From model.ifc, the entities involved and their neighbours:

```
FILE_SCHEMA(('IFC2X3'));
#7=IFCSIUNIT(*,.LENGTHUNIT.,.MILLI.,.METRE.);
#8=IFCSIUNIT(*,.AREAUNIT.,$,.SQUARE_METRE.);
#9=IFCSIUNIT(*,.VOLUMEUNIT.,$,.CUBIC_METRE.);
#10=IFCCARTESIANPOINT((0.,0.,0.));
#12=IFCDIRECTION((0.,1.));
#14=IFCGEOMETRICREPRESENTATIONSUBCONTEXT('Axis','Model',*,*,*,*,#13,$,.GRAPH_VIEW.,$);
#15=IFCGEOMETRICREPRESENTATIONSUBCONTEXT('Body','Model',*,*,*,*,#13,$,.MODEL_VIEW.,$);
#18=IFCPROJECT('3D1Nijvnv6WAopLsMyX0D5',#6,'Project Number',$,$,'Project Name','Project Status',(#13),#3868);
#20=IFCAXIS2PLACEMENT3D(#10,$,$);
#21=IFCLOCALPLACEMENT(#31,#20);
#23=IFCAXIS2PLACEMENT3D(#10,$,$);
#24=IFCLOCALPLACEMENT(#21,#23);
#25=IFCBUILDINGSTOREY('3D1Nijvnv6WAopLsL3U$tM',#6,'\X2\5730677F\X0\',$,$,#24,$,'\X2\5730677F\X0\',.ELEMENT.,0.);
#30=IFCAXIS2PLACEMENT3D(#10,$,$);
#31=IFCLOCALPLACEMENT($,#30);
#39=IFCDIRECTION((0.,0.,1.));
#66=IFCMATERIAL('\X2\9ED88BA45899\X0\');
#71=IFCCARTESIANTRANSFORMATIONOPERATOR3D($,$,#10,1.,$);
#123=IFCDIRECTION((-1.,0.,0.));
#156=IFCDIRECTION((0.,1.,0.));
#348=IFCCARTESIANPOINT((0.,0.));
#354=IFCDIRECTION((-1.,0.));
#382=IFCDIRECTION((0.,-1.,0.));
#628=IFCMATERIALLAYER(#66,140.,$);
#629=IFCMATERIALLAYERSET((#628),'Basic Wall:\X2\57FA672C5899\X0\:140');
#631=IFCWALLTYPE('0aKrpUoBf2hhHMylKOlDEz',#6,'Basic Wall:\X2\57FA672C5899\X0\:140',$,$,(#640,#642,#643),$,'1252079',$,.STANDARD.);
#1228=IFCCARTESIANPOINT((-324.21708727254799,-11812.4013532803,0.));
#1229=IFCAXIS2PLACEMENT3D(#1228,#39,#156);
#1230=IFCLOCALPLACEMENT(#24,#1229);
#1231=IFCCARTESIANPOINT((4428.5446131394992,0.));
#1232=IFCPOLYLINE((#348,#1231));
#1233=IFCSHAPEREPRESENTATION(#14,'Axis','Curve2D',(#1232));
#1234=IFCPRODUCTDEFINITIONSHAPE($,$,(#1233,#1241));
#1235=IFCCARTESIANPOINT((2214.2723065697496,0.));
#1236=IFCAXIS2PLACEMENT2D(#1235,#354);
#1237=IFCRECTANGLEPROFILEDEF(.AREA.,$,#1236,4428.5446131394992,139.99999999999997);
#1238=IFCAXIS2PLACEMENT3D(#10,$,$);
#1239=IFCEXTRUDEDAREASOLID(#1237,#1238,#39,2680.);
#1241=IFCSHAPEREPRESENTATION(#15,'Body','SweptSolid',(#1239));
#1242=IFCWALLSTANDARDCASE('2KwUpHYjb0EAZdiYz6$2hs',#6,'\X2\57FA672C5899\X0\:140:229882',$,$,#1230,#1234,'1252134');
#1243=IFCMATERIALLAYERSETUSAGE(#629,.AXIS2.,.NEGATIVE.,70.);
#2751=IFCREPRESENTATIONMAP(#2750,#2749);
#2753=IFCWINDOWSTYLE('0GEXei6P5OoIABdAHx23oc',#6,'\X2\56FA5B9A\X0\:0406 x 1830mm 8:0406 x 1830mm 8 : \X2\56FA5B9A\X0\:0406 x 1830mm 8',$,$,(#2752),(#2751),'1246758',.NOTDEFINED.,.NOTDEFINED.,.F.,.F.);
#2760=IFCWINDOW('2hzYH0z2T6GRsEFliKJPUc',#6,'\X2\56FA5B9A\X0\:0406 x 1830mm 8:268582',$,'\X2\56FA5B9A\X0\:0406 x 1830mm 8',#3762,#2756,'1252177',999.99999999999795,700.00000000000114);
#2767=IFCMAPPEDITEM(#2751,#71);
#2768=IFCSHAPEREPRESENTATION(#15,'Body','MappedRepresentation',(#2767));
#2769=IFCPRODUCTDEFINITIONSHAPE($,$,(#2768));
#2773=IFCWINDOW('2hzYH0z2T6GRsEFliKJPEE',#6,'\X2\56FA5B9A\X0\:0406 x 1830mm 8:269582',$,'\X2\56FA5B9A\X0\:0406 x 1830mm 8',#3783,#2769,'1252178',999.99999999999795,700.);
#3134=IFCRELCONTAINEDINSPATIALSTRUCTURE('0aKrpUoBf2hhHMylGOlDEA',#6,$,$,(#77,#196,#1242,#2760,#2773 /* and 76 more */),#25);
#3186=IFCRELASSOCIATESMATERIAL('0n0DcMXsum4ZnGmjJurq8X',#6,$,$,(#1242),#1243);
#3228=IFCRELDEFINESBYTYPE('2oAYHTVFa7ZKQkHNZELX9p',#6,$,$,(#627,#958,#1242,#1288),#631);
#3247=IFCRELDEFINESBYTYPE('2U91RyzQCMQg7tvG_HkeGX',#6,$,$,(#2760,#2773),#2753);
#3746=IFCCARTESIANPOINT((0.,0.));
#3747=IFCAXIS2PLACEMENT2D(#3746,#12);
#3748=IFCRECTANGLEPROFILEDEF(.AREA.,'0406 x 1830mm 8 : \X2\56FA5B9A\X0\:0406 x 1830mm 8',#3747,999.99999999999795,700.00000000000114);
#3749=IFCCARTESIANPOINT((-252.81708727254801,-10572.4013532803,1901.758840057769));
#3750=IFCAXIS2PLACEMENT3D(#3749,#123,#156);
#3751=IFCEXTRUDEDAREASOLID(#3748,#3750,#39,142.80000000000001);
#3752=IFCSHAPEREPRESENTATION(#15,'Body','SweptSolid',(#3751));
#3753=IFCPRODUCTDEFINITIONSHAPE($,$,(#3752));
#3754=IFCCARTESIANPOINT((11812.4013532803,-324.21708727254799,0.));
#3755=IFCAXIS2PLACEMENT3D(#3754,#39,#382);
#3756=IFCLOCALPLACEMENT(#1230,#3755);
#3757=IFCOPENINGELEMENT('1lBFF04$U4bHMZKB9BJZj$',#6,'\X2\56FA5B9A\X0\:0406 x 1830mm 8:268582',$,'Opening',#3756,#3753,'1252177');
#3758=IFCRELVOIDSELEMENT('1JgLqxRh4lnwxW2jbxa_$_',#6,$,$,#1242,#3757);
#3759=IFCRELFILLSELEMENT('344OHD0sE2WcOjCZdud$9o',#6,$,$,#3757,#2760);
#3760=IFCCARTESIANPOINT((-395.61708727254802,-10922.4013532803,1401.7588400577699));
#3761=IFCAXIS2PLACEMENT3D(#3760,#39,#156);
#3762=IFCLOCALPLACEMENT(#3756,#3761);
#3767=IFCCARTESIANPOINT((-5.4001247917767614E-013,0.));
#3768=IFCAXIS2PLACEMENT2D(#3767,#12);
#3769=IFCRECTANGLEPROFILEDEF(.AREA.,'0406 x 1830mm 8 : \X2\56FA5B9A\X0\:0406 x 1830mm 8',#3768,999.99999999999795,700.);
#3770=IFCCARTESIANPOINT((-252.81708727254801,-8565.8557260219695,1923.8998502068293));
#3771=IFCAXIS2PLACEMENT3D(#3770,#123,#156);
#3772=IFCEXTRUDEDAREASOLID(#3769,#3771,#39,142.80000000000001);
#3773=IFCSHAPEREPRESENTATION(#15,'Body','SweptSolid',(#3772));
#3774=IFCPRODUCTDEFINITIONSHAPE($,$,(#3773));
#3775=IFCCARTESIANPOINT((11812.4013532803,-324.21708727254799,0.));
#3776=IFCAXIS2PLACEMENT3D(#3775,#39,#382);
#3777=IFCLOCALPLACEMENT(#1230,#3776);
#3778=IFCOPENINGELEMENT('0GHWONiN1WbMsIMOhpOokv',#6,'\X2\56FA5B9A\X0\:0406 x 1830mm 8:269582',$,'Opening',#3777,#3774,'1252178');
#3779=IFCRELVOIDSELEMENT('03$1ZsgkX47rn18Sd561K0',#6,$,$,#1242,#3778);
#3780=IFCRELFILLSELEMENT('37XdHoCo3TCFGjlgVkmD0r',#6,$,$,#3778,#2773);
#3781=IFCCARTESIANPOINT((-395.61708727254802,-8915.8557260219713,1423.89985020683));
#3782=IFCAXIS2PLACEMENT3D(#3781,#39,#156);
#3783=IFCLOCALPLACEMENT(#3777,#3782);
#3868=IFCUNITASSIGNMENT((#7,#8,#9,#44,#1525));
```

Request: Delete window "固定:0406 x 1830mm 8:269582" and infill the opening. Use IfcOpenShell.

```python
import ifcopenshell
import ifcopenshell.api.feature
import ifcopenshell.api.root
import ifcopenshell.geom
import ifcopenshell.util.shape

model = ifcopenshell.open("model.ifc")
settings = ifcopenshell.geom.settings()


def volume(element):
    """Net volume in cubic metres, openings subtracted."""
    shape = ifcopenshell.geom.create_shape(settings, element)
    return ifcopenshell.util.shape.get_volume(shape.geometry)


window = model.by_guid("2hzYH0z2T6GRsEFliKJPEE")
opening = window.FillsVoids[0].RelatingOpeningElement
wall = opening.VoidsElements[0].RelatingBuildingElement
before = volume(wall)

ifcopenshell.api.root.remove_product(model, product=window)
ifcopenshell.api.feature.remove_feature(model, feature=opening)

after = volume(wall)

print(f"wall volume {before:.3f} -> {after:.3f} m3")

model.write("model_rev.ifc")
```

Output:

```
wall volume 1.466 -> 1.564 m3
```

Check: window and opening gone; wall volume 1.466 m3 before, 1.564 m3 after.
